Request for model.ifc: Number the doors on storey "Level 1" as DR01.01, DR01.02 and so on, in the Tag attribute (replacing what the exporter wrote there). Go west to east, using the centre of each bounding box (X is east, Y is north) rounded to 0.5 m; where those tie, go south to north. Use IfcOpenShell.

First a look at what the model holds.

```python
import ifcopenshell
import ifcopenshell.util.element
import ifcopenshell.util.placement

model = ifcopenshell.open("model.ifc")
print(model.schema)
storey = next(s for s in model.by_type("IfcBuildingStorey") if s.Name == "Level 1")
doors = [e for e in ifcopenshell.util.element.get_decomposition(storey) if e.is_a("IfcDoor")]
for e in sorted(doors, key=lambda e: e.id()):
    origin = ifcopenshell.util.placement.get_local_placement(e.ObjectPlacement)[:3, 3]
    print(e.id(), e.Tag, e.Name, origin.round(2) + 0.0, sep=" | ")
```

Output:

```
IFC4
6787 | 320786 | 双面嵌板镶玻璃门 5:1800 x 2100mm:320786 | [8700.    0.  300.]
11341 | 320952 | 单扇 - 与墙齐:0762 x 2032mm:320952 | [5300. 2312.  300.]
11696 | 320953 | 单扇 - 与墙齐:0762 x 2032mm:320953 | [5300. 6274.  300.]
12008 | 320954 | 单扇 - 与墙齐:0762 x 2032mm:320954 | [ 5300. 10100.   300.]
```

```python
import ifcopenshell
import ifcopenshell.geom
import ifcopenshell.util.element
import ifcopenshell.util.shape

model = ifcopenshell.open("model.ifc")
settings = ifcopenshell.geom.settings()
settings.set("use-world-coords", True)


def centre(element):
    shape = ifcopenshell.geom.create_shape(settings, element)
    return ifcopenshell.util.shape.get_bbox_centroid(shape.geometry)


storey = next(s for s in model.by_type("IfcBuildingStorey") if s.Name == "Level 1")
doors = [e for e in ifcopenshell.util.element.get_decomposition(storey) if e.is_a("IfcDoor")]

# Insertion points can sit at a corner or the storey origin, so sort by the geometry (in metres).
centres = {e: centre(e) for e in doors}
doors.sort(key=lambda e: (round(centres[e][0] / 0.5), centres[e][1]))

for i, e in enumerate(doors, start=1):
    number = f"DR01.{i:02d}"
    e.Tag = number
    print(e.id(), number)

model.write("model_v2.ifc")
```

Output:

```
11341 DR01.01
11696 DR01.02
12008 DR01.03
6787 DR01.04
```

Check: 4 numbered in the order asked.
